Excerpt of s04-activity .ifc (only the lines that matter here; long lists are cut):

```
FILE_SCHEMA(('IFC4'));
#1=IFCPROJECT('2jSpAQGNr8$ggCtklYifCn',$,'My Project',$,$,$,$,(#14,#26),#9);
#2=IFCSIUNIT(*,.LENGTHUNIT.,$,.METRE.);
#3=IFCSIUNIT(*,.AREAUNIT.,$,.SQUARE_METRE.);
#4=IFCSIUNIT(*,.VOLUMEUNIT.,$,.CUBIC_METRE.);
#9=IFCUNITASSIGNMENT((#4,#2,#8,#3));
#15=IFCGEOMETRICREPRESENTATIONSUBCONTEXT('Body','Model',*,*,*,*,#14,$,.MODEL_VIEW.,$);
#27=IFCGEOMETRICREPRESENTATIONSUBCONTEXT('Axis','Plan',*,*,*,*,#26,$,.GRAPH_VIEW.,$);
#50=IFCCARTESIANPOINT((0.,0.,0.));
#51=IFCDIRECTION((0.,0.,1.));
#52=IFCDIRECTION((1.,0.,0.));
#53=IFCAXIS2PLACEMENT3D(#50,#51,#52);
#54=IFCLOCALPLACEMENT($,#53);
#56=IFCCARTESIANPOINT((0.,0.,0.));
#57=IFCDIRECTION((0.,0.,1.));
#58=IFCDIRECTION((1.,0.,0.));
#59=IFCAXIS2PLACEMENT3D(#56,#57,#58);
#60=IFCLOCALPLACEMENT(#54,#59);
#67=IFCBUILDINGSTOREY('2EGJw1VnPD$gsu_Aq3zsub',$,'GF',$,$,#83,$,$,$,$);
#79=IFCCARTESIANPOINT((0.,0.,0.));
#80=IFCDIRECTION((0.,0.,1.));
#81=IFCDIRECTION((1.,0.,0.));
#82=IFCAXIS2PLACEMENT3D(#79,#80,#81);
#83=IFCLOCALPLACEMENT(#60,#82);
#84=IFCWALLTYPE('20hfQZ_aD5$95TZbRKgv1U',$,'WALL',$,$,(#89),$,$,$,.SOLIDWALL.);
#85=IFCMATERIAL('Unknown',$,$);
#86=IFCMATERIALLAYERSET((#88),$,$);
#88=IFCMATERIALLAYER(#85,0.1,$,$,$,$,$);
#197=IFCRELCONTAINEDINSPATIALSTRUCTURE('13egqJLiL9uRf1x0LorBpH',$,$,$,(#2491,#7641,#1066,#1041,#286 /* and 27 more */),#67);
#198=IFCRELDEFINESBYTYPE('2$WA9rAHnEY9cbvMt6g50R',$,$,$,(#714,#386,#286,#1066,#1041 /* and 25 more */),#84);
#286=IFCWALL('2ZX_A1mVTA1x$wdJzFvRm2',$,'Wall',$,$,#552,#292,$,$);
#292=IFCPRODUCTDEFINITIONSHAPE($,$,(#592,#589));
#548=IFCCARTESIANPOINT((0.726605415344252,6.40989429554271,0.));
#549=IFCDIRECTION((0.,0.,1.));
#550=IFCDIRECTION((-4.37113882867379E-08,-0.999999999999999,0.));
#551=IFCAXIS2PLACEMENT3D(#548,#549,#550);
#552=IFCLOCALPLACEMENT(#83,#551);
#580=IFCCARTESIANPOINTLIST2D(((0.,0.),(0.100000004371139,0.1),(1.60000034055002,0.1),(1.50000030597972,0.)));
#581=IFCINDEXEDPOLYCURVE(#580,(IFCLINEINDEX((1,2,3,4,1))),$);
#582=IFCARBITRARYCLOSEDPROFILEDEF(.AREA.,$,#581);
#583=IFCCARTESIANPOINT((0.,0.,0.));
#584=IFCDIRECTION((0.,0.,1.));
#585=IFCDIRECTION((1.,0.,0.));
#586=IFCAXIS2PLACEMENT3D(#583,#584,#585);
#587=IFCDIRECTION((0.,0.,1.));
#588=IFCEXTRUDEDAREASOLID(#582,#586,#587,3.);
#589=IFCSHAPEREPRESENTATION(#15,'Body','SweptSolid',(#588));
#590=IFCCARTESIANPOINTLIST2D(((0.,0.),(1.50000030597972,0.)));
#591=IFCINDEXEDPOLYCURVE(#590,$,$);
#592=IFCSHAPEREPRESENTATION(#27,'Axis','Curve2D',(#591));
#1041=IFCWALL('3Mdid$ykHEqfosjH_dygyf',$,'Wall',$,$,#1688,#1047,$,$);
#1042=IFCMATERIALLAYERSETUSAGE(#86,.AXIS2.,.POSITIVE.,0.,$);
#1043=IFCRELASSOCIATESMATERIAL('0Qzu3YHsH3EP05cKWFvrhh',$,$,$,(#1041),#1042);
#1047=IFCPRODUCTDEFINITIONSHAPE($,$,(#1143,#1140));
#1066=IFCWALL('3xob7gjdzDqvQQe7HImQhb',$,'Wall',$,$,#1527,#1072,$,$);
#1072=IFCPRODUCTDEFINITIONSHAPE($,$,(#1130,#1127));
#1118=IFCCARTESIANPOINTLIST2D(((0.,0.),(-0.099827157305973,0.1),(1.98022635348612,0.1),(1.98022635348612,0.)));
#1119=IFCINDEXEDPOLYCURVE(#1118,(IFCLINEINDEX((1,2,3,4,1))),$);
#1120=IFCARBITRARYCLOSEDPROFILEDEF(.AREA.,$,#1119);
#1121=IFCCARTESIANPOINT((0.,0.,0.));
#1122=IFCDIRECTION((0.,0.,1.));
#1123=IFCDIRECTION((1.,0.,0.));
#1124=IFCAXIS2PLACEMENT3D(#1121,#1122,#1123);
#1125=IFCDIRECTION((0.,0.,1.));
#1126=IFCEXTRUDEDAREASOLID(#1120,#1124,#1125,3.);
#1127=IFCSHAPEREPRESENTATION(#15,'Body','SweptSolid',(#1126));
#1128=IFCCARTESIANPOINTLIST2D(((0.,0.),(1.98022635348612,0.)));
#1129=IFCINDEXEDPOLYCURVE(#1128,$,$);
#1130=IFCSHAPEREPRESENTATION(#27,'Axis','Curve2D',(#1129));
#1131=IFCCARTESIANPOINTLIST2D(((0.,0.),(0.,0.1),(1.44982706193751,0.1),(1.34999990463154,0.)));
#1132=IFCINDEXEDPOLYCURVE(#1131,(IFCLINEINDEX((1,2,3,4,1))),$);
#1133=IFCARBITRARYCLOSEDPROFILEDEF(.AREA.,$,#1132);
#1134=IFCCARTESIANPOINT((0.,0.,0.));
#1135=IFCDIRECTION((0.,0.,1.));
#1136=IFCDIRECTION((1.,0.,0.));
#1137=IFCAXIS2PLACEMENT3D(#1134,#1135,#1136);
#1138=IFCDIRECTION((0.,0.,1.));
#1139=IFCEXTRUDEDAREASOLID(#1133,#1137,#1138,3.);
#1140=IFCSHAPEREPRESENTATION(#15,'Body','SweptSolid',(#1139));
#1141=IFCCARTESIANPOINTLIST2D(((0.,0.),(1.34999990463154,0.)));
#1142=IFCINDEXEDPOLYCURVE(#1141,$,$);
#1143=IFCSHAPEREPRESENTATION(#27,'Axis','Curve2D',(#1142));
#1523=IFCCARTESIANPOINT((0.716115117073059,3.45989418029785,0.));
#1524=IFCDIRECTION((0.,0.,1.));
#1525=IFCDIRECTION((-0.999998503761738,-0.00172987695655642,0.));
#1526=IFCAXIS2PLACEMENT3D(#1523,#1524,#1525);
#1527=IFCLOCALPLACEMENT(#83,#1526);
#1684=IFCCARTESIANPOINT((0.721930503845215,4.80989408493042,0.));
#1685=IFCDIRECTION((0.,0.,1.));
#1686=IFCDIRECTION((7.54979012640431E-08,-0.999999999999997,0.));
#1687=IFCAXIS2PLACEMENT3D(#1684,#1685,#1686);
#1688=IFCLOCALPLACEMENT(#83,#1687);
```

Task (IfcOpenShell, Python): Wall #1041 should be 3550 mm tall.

```python
import ifcopenshell
import ifcopenshell.geom
import ifcopenshell.util.representation
import ifcopenshell.util.shape
import ifcopenshell.util.unit

model = ifcopenshell.open("s04-activity .ifc")
unit_scale = ifcopenshell.util.unit.calculate_unit_scale(model)
settings = ifcopenshell.geom.settings()


def volume(element):
    """Net volume in cubic metres, openings subtracted."""
    shape = ifcopenshell.geom.create_shape(settings, element)
    return ifcopenshell.util.shape.get_volume(shape.geometry)


wall = model.by_guid("3Mdid$ykHEqfosjH_dygyf")
before = volume(wall)

body = ifcopenshell.util.representation.get_representation(wall, "Model", "Body")
solid = body.Items[0]
old_height = solid.Depth
solid.Depth = 3.55 / unit_scale
after = volume(wall)

print(f"height {old_height:g} -> {solid.Depth:g}, volume {before:.3f} -> {after:.3f} m3")

model.write("s04-activity -out.ifc")
```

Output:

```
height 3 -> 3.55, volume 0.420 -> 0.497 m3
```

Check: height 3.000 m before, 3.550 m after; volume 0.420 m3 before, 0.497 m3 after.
